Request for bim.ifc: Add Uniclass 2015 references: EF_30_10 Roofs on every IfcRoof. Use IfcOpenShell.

First a look at what the model holds.

```python
import ifcopenshell

model = ifcopenshell.open("bim.ifc")
print(model.schema)
print("classifications:", [c.Name for c in model.by_type("IfcClassification")])
for ifc_class in ("IfcDoor", "IfcRoof", "IfcStair", "IfcWall", "IfcWindow"):
    print(ifc_class, len(model.by_type(ifc_class)))
```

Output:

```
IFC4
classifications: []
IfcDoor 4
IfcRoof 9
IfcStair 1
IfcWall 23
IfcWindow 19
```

```python
import ifcopenshell
import ifcopenshell.api.classification

model = ifcopenshell.open("bim.ifc")

system = ifcopenshell.api.classification.add_classification(model, classification="Uniclass 2015")

codes = {
    "IfcRoof": ("EF_30_10", "Roofs"),
}
for ifc_class, (code, name) in codes.items():
    products = model.by_type(ifc_class)
    ifcopenshell.api.classification.add_reference(
        model, products=products, classification=system, identification=code, name=name
    )
    print(code, len(products))

model.write("bim-out.ifc")
```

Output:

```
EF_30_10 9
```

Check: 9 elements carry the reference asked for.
